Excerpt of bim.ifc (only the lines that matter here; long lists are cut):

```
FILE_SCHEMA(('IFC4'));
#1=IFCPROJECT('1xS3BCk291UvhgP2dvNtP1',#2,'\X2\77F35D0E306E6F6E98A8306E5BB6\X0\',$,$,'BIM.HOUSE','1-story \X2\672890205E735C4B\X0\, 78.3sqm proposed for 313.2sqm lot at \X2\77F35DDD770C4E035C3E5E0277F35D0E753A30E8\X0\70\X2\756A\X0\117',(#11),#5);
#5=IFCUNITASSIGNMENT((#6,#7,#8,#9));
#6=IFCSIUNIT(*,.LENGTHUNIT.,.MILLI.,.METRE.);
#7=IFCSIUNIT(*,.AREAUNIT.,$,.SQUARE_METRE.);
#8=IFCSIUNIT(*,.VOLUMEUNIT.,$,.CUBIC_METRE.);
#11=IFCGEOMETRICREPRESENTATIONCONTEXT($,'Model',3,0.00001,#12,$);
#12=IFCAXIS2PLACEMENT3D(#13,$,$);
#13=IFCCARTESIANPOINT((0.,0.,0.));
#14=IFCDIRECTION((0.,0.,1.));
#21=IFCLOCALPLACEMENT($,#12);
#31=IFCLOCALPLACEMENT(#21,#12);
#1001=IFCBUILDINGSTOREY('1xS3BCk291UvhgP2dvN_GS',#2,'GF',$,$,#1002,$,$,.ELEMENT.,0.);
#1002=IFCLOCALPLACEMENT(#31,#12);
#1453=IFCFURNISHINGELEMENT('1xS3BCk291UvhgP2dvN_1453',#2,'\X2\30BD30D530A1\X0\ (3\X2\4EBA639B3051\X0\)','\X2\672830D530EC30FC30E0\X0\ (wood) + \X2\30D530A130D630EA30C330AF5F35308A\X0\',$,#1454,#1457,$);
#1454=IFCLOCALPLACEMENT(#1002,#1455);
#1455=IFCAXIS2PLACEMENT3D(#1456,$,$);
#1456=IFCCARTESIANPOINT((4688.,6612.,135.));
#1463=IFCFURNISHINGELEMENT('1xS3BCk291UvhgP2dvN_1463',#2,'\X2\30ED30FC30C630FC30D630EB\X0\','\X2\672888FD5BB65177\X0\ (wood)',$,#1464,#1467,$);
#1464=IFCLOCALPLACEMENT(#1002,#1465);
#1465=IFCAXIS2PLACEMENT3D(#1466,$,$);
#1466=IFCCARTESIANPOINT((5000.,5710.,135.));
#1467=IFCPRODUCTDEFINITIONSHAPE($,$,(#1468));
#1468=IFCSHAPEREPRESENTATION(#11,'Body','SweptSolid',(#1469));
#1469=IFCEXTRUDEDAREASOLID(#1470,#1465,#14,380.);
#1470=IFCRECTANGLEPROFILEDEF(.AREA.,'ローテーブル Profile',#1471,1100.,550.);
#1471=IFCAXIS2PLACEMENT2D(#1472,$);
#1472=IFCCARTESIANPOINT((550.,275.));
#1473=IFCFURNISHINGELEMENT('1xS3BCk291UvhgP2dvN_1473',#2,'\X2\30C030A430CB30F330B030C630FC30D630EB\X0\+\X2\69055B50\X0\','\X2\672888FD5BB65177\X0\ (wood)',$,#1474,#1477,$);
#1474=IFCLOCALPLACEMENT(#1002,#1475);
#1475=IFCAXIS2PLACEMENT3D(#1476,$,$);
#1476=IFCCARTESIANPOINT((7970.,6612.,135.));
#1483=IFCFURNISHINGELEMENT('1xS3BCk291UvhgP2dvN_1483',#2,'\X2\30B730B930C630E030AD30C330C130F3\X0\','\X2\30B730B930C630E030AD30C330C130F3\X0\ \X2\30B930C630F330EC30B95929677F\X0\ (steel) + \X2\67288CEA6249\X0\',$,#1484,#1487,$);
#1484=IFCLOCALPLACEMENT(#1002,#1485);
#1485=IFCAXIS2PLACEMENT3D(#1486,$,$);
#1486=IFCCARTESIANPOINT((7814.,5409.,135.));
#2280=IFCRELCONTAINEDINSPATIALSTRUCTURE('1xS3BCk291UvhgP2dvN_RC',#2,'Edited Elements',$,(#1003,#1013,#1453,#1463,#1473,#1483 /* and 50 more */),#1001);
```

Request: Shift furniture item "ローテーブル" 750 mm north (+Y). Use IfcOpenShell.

```python
import ifcopenshell
import ifcopenshell.api.geometry
import ifcopenshell.util.placement
import ifcopenshell.util.unit

model = ifcopenshell.open("bim.ifc")
unit_scale = ifcopenshell.util.unit.calculate_unit_scale(model)

item = model.by_guid("1xS3BCk291UvhgP2dvN_1463")
matrix = ifcopenshell.util.placement.get_local_placement(item.ObjectPlacement)
matrix[1, 3] += 0.75 / unit_scale
ifcopenshell.api.geometry.edit_object_placement(model, product=item, matrix=matrix, is_si=False)

print(ifcopenshell.util.placement.get_local_placement(item.ObjectPlacement).round(3) + 0.0)

model.write("bim_v2.ifc")
```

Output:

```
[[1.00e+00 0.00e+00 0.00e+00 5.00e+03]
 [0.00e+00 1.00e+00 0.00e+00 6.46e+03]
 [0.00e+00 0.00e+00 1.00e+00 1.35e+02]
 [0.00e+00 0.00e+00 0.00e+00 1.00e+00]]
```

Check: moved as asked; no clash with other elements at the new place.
